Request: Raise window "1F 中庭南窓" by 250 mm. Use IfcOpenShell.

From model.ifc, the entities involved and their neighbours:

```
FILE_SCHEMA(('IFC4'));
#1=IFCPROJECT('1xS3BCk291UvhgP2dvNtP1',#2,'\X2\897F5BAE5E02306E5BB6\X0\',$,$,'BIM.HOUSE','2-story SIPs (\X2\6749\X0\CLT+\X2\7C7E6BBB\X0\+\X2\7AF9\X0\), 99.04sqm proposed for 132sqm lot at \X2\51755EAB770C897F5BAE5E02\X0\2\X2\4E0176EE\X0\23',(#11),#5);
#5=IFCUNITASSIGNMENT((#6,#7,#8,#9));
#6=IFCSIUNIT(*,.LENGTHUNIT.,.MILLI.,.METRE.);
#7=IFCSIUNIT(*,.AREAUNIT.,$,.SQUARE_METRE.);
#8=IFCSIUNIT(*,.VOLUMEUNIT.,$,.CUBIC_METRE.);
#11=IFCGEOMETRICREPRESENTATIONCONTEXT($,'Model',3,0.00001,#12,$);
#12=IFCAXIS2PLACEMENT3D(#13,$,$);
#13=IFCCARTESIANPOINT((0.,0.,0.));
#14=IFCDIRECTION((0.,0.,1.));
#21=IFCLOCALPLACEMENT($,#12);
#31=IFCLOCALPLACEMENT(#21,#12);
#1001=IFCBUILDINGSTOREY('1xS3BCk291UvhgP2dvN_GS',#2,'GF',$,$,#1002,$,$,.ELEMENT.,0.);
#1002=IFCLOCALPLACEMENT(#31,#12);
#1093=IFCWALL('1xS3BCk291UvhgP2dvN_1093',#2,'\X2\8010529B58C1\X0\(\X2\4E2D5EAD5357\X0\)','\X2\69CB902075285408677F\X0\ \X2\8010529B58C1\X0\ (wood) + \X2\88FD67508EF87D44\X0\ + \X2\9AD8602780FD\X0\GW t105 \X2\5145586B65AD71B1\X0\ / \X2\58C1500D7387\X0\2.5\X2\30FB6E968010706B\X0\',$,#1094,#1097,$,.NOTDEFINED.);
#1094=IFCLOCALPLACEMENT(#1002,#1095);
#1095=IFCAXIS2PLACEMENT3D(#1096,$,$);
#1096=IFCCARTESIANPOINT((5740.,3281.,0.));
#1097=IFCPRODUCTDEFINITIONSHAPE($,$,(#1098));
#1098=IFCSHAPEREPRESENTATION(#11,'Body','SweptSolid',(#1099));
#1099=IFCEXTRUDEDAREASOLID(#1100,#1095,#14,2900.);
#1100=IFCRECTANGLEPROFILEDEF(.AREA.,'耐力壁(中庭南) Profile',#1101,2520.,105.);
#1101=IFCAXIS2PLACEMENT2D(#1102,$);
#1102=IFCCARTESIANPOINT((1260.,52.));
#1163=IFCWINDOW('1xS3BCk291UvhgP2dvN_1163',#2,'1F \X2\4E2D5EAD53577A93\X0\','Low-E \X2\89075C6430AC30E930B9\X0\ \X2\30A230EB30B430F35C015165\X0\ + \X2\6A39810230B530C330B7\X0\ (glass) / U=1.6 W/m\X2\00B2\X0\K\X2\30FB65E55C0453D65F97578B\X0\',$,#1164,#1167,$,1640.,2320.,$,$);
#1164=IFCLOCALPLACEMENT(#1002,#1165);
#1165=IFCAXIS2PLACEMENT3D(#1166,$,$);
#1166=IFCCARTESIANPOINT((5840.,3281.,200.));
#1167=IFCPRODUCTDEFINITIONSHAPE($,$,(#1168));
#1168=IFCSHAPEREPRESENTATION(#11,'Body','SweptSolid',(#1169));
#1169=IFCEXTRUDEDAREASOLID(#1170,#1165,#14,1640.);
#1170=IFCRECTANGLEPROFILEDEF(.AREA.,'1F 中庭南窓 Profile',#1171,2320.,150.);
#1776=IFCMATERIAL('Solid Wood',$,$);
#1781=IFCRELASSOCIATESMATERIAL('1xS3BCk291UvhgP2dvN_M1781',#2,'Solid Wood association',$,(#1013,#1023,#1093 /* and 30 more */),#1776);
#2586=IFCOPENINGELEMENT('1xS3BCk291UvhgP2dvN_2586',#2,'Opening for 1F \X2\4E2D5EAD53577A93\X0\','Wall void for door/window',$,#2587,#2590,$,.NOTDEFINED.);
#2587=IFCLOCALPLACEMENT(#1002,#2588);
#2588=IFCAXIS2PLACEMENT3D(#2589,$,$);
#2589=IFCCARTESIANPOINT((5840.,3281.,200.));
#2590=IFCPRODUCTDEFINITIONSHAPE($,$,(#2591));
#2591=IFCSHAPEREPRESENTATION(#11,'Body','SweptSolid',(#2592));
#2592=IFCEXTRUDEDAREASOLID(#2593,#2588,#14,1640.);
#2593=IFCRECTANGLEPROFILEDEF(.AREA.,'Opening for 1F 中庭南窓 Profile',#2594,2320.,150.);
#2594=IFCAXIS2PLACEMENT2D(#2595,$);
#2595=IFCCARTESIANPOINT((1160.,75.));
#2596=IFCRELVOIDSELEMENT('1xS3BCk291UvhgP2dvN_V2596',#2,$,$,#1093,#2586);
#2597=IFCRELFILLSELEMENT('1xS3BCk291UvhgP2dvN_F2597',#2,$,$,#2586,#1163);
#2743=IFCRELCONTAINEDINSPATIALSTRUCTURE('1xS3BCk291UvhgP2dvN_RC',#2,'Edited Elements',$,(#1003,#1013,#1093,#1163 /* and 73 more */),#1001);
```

```python
import numpy as np
import ifcopenshell
import ifcopenshell.api.geometry
import ifcopenshell.util.placement
import ifcopenshell.util.unit

model = ifcopenshell.open("model.ifc")
unit_scale = ifcopenshell.util.unit.calculate_unit_scale(model)

window = model.by_guid("1xS3BCk291UvhgP2dvN_1163")
opening = window.FillsVoids[0].RelatingOpeningElement
dz = 0.25 / unit_scale

shift = np.array([0.0, 0.0, dz])
# The window is not placed relative to its opening, so move both.
for product in (opening, window):
    matrix = ifcopenshell.util.placement.get_local_placement(product.ObjectPlacement)
    matrix[:3, 3] += shift
    ifcopenshell.api.geometry.edit_object_placement(model, product=product, matrix=matrix, is_si=False)

print(f"moved by {dz * unit_scale:+.3f} m")

model.write("model_updated.ifc")
```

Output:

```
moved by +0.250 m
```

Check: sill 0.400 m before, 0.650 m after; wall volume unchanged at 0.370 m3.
